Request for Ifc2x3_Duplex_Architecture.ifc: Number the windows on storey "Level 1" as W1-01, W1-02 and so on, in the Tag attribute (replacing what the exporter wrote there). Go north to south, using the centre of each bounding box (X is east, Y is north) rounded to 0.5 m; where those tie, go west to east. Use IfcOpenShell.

First a look at what the model holds.

```python
import ifcopenshell
import ifcopenshell.util.element
import ifcopenshell.util.placement

model = ifcopenshell.open("Ifc2x3_Duplex_Architecture.ifc")
print(model.schema)
storey = next(s for s in model.by_type("IfcBuildingStorey") if s.Name == "Level 1")
windows = [e for e in ifcopenshell.util.element.get_decomposition(storey) if e.is_a("IfcWindow")]
for e in sorted(windows, key=lambda e: e.id()):
    origin = ifcopenshell.util.placement.get_local_placement(e.ObjectPlacement)[:3, 3]
    print(e.id(), e.Tag, e.Name, origin.round(2) + 0.0, sep=" | ")
```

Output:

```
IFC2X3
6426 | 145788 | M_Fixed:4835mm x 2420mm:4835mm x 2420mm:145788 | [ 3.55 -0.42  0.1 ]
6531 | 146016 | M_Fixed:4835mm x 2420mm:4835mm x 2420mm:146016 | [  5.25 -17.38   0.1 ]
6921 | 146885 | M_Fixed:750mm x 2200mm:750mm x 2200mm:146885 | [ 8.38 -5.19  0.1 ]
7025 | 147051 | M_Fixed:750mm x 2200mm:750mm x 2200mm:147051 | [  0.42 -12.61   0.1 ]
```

```python
import ifcopenshell
import ifcopenshell.geom
import ifcopenshell.util.element
import ifcopenshell.util.shape

model = ifcopenshell.open("Ifc2x3_Duplex_Architecture.ifc")
settings = ifcopenshell.geom.settings()
settings.set("use-world-coords", True)


def centre(element):
    shape = ifcopenshell.geom.create_shape(settings, element)
    return ifcopenshell.util.shape.get_bbox_centroid(shape.geometry)


storey = next(s for s in model.by_type("IfcBuildingStorey") if s.Name == "Level 1")
windows = [e for e in ifcopenshell.util.element.get_decomposition(storey) if e.is_a("IfcWindow")]

# Insertion points can sit at a corner or the storey origin, so sort by the geometry (in metres).
centres = {e: centre(e) for e in windows}
windows.sort(key=lambda e: (-round(centres[e][1] / 0.5), centres[e][0]))

for i, e in enumerate(windows, start=1):
    number = f"W1-{i:02d}"
    e.Tag = number
    print(e.id(), number)

model.write("Ifc2x3_Duplex_Architecture-out.ifc")
```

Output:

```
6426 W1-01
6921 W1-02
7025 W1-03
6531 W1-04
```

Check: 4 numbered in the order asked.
